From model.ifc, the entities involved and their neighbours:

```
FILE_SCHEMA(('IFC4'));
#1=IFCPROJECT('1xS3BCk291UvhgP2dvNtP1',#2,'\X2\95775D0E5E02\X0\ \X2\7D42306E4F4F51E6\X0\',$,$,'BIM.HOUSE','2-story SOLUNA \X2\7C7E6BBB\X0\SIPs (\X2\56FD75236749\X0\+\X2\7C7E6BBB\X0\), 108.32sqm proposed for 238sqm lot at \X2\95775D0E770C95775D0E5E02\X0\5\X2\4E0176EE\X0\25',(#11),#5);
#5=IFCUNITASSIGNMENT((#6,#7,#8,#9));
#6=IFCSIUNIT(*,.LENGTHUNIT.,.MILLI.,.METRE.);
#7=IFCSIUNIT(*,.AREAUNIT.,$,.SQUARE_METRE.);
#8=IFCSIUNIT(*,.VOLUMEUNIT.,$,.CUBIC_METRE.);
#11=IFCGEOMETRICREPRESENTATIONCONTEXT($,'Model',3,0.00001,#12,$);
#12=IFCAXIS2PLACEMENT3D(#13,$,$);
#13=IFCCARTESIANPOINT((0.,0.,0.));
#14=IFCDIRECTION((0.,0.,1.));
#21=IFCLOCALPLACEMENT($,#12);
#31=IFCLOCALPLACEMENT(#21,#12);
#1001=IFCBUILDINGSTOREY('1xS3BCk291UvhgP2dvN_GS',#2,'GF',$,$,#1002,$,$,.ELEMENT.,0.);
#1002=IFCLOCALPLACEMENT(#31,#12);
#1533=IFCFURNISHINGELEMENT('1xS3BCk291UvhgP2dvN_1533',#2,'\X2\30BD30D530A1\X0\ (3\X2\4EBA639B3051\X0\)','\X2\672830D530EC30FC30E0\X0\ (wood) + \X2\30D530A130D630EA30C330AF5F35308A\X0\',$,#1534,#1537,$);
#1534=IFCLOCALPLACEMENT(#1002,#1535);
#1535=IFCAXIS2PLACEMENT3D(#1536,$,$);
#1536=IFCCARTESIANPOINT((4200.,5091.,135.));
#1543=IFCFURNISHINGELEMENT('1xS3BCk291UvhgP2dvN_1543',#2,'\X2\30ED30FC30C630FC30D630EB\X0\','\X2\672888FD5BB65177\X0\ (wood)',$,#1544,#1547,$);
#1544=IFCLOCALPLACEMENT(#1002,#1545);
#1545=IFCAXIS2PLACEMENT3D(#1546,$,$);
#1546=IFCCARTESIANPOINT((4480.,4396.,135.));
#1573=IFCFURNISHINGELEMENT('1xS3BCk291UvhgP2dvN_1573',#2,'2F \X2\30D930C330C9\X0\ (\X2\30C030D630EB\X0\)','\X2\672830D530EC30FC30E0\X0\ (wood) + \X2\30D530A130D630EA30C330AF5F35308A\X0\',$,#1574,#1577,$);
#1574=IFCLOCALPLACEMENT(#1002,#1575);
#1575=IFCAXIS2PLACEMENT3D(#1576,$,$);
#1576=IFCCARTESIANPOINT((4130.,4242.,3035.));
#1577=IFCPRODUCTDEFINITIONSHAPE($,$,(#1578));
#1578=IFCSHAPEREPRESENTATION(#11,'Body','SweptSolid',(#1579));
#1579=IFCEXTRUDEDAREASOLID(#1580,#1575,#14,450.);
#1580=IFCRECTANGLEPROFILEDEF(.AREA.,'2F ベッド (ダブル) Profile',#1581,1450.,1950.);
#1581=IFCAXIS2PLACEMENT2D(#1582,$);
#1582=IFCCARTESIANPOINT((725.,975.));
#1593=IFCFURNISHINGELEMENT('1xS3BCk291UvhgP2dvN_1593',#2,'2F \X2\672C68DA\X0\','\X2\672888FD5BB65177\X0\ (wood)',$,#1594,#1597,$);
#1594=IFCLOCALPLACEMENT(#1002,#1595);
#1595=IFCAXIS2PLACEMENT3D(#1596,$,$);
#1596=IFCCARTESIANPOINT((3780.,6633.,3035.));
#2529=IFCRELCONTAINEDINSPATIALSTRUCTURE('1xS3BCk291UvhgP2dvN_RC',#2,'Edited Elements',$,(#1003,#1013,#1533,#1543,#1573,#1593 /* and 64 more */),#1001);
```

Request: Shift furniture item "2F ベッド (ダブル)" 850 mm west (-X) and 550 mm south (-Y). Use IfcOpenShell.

```python
import ifcopenshell
import ifcopenshell.api.geometry
import ifcopenshell.util.placement
import ifcopenshell.util.unit

model = ifcopenshell.open("model.ifc")
unit_scale = ifcopenshell.util.unit.calculate_unit_scale(model)

item = model.by_guid("1xS3BCk291UvhgP2dvN_1573")
matrix = ifcopenshell.util.placement.get_local_placement(item.ObjectPlacement)
matrix[0, 3] -= 0.85 / unit_scale
matrix[1, 3] -= 0.55 / unit_scale
ifcopenshell.api.geometry.edit_object_placement(model, product=item, matrix=matrix, is_si=False)

print(ifcopenshell.util.placement.get_local_placement(item.ObjectPlacement).round(3) + 0.0)

model.write("model_rev.ifc")
```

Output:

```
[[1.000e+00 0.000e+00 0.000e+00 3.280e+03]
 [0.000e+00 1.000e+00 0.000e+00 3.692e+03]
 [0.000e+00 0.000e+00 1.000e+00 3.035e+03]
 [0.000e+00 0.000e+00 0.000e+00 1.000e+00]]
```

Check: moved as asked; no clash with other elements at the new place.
